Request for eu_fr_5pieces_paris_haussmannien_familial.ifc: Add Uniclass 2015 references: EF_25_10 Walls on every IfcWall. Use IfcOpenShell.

First a look at what the model holds.

```python
import ifcopenshell

model = ifcopenshell.open("eu_fr_5pieces_paris_haussmannien_familial.ifc")
print(model.schema)
print("classifications:", [c.Name for c in model.by_type("IfcClassification")])
for ifc_class in ("IfcDoor", "IfcRoof", "IfcStair", "IfcWall", "IfcWindow"):
    print(ifc_class, len(model.by_type(ifc_class)))
```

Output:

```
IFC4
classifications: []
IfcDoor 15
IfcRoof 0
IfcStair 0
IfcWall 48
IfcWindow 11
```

```python
import ifcopenshell
import ifcopenshell.api.classification

model = ifcopenshell.open("eu_fr_5pieces_paris_haussmannien_familial.ifc")

system = ifcopenshell.api.classification.add_classification(model, classification="Uniclass 2015")

codes = {
    "IfcWall": ("EF_25_10", "Walls"),
}
for ifc_class, (code, name) in codes.items():
    products = model.by_type(ifc_class)
    ifcopenshell.api.classification.add_reference(
        model, products=products, classification=system, identification=code, name=name
    )
    print(code, len(products))

model.write("eu_fr_5pieces_paris_haussmannien_familial-out.ifc")
```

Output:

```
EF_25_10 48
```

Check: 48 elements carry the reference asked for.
